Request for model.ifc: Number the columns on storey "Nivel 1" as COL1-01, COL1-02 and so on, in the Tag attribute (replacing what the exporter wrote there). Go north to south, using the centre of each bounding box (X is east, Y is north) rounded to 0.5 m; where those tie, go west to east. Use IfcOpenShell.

First a look at what the model holds.

```python
import ifcopenshell
import ifcopenshell.util.element
import ifcopenshell.util.placement

model = ifcopenshell.open("model.ifc")
print(model.schema)
storey = next(s for s in model.by_type("IfcBuildingStorey") if s.Name == "Nivel 1")
columns = [e for e in ifcopenshell.util.element.get_decomposition(storey) if e.is_a("IfcColumn")]
for e in sorted(columns, key=lambda e: e.id()):
    origin = ifcopenshell.util.placement.get_local_placement(e.ObjectPlacement)[:3, 3]
    print(e.id(), e.Tag, e.Name, origin.round(2) + 0.0, sep=" | ")
```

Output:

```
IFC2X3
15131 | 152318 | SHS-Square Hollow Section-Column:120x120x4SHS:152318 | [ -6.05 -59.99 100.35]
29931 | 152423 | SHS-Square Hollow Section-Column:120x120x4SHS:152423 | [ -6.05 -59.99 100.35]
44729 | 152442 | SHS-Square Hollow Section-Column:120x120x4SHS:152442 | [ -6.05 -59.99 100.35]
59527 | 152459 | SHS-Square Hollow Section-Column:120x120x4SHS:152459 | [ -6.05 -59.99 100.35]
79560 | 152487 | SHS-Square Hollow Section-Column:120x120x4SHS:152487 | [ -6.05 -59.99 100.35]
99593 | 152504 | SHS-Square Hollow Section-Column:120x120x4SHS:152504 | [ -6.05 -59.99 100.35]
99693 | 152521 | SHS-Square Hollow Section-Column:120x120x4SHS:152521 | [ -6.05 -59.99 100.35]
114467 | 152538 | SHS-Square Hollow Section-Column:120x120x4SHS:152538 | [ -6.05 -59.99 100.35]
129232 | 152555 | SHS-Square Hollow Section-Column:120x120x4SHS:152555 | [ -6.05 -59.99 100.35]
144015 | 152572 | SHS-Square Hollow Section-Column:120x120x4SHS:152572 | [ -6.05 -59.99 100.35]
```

```python
import ifcopenshell
import ifcopenshell.geom
import ifcopenshell.util.element
import ifcopenshell.util.shape

model = ifcopenshell.open("model.ifc")
settings = ifcopenshell.geom.settings()
settings.set("use-world-coords", True)


def centre(element):
    shape = ifcopenshell.geom.create_shape(settings, element)
    return ifcopenshell.util.shape.get_bbox_centroid(shape.geometry)


storey = next(s for s in model.by_type("IfcBuildingStorey") if s.Name == "Nivel 1")
columns = [e for e in ifcopenshell.util.element.get_decomposition(storey) if e.is_a("IfcColumn")]

# Insertion points can sit at a corner or the storey origin, so sort by the geometry (in metres).
centres = {e: centre(e) for e in columns}
columns.sort(key=lambda e: (-round(centres[e][1] / 0.5), centres[e][0]))

for i, e in enumerate(columns, start=1):
    number = f"COL1-{i:02d}"
    e.Tag = number
    print(e.id(), number)

model.write("model_v2.ifc")
```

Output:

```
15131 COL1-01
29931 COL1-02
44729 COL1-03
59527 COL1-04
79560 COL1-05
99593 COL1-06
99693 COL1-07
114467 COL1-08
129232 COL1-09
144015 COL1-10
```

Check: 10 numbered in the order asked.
